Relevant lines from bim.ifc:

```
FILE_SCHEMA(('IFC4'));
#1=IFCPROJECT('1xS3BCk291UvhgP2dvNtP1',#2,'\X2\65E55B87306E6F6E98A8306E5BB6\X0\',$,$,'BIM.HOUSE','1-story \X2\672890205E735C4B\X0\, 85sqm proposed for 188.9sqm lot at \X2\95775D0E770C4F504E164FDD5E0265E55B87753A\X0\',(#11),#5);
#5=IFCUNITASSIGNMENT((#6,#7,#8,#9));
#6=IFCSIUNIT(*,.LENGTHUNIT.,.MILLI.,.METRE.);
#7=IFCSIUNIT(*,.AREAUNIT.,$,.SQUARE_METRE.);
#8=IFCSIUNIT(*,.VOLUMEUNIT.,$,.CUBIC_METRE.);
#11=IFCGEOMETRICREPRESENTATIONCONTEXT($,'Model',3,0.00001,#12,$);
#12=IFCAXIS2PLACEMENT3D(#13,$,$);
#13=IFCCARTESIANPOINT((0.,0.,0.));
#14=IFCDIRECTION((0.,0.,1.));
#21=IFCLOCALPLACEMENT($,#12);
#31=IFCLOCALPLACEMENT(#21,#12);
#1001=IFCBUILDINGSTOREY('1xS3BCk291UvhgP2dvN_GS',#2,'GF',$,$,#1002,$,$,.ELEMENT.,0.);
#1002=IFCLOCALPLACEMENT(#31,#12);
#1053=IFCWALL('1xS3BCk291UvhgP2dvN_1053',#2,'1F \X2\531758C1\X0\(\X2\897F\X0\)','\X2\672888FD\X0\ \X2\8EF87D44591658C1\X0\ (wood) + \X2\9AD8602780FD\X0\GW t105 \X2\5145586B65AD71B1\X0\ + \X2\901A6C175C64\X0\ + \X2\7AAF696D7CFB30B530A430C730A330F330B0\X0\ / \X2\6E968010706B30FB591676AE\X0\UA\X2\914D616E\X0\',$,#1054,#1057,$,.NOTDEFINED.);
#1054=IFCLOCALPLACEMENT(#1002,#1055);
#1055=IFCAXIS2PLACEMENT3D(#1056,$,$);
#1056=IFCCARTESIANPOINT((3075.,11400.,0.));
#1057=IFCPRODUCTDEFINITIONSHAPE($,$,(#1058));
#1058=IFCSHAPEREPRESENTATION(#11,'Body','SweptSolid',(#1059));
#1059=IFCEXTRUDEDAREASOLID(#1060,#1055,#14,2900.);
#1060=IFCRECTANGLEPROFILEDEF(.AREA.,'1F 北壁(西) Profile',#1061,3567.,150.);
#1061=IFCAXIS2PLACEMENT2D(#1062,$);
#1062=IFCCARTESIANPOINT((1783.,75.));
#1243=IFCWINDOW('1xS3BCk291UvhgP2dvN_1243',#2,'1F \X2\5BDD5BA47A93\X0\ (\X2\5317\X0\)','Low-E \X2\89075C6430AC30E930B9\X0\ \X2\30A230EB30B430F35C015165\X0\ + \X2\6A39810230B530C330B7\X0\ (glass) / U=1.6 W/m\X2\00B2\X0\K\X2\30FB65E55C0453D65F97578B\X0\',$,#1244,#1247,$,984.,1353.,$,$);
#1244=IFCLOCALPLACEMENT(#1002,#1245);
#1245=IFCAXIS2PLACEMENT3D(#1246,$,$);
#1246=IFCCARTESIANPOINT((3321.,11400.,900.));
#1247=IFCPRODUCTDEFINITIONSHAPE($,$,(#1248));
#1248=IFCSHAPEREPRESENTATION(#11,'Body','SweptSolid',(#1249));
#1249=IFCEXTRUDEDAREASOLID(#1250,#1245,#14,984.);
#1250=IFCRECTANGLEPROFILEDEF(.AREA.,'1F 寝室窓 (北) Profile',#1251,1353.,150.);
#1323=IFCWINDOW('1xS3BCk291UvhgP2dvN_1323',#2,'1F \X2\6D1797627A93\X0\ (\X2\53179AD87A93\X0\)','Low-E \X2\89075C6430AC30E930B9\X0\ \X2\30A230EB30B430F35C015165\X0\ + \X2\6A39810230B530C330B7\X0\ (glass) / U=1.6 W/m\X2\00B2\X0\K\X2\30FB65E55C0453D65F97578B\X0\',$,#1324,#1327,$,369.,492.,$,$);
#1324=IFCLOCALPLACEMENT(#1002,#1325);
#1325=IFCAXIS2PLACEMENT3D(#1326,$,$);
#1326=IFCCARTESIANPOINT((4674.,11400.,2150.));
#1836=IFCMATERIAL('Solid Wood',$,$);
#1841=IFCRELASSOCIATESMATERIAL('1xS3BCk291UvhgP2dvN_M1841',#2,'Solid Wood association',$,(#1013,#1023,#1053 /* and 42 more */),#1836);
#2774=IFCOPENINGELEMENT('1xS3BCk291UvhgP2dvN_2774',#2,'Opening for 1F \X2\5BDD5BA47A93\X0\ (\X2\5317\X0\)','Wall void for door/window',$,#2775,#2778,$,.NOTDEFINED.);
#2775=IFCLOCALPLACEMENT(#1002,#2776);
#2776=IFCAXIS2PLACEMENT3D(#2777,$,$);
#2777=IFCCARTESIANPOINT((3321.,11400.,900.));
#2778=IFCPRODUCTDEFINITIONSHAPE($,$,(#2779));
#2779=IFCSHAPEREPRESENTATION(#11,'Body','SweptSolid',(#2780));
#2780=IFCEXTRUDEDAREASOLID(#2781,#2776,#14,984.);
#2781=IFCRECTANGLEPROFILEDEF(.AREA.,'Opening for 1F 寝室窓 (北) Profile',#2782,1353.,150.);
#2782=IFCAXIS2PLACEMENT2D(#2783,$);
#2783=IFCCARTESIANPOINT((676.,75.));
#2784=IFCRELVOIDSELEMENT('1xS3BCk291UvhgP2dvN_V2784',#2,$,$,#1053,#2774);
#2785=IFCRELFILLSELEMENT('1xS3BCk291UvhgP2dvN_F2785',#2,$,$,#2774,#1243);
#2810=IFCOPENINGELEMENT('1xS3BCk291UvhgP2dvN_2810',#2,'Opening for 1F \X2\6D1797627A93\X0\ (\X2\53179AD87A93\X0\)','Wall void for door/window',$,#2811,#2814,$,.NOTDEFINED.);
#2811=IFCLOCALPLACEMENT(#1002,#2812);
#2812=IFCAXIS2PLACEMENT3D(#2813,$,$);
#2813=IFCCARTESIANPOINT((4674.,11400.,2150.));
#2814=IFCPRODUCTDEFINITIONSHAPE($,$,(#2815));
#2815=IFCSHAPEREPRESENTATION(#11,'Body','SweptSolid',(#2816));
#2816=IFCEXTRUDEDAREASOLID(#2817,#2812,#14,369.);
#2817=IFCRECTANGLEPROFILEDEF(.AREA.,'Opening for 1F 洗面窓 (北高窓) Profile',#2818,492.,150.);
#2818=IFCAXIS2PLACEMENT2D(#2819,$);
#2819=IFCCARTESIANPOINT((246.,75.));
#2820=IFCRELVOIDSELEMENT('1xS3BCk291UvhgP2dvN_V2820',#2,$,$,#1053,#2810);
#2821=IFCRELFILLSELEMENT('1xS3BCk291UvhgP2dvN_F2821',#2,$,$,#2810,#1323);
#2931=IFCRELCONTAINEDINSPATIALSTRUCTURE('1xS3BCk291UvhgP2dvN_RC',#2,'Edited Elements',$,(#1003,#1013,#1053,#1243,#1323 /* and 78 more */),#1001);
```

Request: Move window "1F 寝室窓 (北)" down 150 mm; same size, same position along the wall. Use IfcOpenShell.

```python
import numpy as np
import ifcopenshell
import ifcopenshell.api.geometry
import ifcopenshell.util.placement
import ifcopenshell.util.unit

model = ifcopenshell.open("bim.ifc")
unit_scale = ifcopenshell.util.unit.calculate_unit_scale(model)

window = model.by_guid("1xS3BCk291UvhgP2dvN_1243")
opening = window.FillsVoids[0].RelatingOpeningElement
dz = -0.15 / unit_scale

shift = np.array([0.0, 0.0, dz])
# The window is not placed relative to its opening, so move both.
for product in (opening, window):
    matrix = ifcopenshell.util.placement.get_local_placement(product.ObjectPlacement)
    matrix[:3, 3] += shift
    ifcopenshell.api.geometry.edit_object_placement(model, product=product, matrix=matrix, is_si=False)

print(f"moved by {dz * unit_scale:+.3f} m")

model.write("bim_updated.ifc")
```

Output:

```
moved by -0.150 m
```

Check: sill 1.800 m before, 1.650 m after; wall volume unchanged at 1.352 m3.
